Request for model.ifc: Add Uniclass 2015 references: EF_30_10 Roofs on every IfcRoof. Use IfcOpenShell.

First a look at what the model holds.

```python
import ifcopenshell

model = ifcopenshell.open("model.ifc")
print(model.schema)
print("classifications:", [c.Name for c in model.by_type("IfcClassification")])
for ifc_class in ("IfcDoor", "IfcRoof", "IfcStair", "IfcWall", "IfcWindow"):
    print(ifc_class, len(model.by_type(ifc_class)))
```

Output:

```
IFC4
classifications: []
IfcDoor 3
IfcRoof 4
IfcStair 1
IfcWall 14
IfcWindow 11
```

```python
import ifcopenshell
import ifcopenshell.api.classification

model = ifcopenshell.open("model.ifc")

system = ifcopenshell.api.classification.add_classification(model, classification="Uniclass 2015")

codes = {
    "IfcRoof": ("EF_30_10", "Roofs"),
}
for ifc_class, (code, name) in codes.items():
    products = model.by_type(ifc_class)
    ifcopenshell.api.classification.add_reference(
        model, products=products, classification=system, identification=code, name=name
    )
    print(code, len(products))

model.write("model_rev.ifc")
```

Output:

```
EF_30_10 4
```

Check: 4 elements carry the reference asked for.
